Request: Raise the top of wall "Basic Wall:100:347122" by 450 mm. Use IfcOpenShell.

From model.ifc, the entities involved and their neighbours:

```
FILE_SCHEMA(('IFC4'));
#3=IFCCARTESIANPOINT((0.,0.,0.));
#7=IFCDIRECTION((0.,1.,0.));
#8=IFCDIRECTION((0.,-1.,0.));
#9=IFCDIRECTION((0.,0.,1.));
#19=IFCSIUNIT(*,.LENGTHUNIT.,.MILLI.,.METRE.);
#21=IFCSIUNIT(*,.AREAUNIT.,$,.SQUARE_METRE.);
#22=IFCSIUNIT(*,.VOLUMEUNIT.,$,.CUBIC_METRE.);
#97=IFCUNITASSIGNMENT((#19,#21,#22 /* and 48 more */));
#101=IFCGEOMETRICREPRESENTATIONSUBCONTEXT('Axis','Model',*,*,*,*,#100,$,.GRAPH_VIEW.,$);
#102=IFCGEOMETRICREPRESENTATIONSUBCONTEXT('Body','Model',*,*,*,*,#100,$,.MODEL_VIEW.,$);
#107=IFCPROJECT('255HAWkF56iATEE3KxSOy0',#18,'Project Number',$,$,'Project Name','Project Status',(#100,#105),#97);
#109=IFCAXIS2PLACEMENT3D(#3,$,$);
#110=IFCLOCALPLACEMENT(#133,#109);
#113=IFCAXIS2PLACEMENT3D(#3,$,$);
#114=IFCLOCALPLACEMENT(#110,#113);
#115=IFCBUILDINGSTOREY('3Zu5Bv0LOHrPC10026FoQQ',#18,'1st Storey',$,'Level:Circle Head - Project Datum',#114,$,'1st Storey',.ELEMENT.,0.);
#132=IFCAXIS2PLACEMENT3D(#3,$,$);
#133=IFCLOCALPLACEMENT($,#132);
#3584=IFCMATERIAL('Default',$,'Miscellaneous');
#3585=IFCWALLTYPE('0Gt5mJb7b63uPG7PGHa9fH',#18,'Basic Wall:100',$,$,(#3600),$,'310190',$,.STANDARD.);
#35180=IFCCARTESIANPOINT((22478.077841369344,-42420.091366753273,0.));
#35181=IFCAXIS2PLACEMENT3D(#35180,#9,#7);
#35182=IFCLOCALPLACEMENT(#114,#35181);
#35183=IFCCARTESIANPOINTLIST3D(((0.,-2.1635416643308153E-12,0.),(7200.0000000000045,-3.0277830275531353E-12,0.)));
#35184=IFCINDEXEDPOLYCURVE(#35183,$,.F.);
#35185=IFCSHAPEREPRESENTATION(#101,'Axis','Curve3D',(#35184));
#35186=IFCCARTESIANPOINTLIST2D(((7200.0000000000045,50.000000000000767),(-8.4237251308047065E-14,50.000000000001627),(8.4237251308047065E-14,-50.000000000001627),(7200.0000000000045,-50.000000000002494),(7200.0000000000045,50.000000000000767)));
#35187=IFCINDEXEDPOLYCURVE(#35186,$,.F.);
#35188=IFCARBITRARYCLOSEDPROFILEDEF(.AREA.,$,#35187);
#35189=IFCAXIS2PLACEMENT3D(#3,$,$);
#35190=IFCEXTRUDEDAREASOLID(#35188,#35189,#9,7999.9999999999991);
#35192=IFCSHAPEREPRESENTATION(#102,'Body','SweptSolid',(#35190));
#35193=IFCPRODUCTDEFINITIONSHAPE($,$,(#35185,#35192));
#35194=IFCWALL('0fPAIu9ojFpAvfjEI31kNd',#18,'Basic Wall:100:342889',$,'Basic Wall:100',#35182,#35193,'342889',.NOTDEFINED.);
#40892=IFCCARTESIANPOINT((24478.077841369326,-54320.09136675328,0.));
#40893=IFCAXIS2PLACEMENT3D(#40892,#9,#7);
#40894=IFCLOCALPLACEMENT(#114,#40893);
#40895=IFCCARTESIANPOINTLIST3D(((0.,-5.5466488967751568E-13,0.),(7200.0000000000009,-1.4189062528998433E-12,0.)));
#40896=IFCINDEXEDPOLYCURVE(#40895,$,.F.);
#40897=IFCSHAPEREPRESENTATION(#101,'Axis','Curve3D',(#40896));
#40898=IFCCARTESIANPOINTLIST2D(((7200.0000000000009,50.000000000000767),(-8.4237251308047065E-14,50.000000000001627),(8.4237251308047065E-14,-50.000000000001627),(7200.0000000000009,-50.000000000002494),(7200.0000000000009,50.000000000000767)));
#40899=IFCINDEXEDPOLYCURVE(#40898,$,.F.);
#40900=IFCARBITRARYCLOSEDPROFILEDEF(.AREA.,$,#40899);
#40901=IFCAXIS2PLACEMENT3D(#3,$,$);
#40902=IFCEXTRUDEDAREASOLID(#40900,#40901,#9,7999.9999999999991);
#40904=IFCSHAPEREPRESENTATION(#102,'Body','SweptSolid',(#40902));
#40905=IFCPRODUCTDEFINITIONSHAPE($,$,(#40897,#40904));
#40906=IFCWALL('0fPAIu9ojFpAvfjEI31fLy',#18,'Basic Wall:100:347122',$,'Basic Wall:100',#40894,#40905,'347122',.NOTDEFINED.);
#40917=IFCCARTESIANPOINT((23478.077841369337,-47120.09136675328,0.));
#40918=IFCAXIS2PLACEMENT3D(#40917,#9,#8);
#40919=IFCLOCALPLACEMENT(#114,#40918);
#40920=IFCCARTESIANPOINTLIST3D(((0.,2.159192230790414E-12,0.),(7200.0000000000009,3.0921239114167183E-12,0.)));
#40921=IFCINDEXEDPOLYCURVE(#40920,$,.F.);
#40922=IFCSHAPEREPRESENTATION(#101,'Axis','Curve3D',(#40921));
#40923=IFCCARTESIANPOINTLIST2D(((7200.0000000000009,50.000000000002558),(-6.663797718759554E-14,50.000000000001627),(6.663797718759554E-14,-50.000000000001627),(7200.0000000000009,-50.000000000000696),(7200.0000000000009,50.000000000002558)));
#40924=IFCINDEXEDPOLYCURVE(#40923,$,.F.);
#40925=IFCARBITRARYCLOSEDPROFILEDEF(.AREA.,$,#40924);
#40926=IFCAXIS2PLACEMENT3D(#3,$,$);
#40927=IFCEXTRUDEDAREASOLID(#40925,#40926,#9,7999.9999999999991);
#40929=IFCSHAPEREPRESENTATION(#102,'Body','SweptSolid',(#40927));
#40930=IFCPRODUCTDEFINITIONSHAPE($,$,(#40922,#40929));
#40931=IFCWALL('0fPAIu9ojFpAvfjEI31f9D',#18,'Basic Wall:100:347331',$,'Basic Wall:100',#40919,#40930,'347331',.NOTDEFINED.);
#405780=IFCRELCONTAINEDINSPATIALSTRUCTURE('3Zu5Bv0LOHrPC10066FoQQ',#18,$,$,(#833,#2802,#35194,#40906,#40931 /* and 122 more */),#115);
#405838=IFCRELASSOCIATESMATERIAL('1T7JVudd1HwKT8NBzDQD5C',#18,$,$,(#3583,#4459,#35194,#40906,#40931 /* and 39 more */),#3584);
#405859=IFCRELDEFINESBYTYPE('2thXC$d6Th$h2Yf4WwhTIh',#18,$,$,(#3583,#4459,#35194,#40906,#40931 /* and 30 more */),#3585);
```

```python
import ifcopenshell
import ifcopenshell.geom
import ifcopenshell.util.representation
import ifcopenshell.util.shape
import ifcopenshell.util.unit

model = ifcopenshell.open("model.ifc")
unit_scale = ifcopenshell.util.unit.calculate_unit_scale(model)
settings = ifcopenshell.geom.settings()


def volume(element):
    """Net volume in cubic metres, openings subtracted."""
    shape = ifcopenshell.geom.create_shape(settings, element)
    return ifcopenshell.util.shape.get_volume(shape.geometry)


wall = model.by_guid("0fPAIu9ojFpAvfjEI31fLy")
before = volume(wall)

body = ifcopenshell.util.representation.get_representation(wall, "Model", "Body")
solid = body.Items[0]
old_height = solid.Depth
solid.Depth += 0.45 / unit_scale
after = volume(wall)

print(f"height {old_height:g} -> {solid.Depth:g}, volume {before:.3f} -> {after:.3f} m3")

model.write("model_rev.ifc")
```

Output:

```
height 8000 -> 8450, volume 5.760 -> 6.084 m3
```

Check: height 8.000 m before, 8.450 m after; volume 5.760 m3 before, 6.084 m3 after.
